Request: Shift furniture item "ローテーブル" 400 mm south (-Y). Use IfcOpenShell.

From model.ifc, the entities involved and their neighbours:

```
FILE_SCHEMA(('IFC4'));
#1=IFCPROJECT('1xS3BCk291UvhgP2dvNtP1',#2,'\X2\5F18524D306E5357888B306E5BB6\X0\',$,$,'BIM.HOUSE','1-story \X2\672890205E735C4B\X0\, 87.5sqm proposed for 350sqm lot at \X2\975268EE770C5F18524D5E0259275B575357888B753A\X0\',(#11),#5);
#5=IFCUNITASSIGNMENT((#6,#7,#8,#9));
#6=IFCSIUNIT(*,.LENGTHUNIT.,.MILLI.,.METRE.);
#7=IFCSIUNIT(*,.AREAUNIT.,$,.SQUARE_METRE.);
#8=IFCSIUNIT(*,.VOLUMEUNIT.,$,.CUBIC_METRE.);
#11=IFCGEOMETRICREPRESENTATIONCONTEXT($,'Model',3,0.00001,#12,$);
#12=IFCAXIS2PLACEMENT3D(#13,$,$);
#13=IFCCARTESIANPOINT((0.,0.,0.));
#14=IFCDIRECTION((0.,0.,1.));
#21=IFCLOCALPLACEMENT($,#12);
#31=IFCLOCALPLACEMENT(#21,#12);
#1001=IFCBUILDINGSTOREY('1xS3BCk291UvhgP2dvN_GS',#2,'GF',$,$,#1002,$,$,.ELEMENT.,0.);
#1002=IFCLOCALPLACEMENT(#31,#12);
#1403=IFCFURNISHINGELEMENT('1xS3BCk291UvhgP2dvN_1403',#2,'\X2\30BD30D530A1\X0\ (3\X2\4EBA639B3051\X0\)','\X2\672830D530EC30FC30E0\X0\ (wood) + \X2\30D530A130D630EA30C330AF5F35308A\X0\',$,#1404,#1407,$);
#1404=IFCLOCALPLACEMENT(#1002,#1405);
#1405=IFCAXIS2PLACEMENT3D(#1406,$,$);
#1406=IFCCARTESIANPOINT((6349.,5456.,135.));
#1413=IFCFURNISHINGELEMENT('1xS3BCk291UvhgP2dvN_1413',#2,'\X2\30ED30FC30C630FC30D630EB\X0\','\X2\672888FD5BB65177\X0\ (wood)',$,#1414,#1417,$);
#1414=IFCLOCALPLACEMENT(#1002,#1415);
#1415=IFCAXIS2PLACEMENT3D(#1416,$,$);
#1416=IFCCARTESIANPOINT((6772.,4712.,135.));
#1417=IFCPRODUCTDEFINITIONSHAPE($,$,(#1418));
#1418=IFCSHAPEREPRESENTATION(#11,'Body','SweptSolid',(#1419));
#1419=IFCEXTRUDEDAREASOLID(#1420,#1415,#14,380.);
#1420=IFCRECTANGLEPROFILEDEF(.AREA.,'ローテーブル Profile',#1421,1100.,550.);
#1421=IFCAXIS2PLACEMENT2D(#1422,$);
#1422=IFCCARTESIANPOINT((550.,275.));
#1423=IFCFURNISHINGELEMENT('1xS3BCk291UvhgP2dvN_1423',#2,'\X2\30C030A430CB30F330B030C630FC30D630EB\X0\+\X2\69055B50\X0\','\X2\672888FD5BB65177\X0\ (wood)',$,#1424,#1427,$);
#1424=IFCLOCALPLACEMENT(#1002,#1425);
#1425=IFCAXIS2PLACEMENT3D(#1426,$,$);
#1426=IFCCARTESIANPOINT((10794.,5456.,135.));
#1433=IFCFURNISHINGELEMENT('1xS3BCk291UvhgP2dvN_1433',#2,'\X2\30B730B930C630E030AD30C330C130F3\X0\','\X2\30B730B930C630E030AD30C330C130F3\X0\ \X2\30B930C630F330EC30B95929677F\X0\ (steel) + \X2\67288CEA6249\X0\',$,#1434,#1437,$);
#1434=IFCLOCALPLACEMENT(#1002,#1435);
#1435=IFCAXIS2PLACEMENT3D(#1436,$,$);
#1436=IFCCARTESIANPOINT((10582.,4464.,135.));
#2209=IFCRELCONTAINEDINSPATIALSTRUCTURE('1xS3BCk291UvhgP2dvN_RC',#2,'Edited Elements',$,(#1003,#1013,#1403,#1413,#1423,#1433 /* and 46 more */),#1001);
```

```python
import ifcopenshell
import ifcopenshell.api.geometry
import ifcopenshell.util.placement

model = ifcopenshell.open("model.ifc")

item = model.by_guid("1xS3BCk291UvhgP2dvN_1413")
matrix = ifcopenshell.util.placement.get_local_placement(item.ObjectPlacement)
matrix[1, 3] -= 400.0
ifcopenshell.api.geometry.edit_object_placement(model, product=item, matrix=matrix, is_si=False)

print(ifcopenshell.util.placement.get_local_placement(item.ObjectPlacement).round(3) + 0.0)

model.write("model_v2.ifc")
```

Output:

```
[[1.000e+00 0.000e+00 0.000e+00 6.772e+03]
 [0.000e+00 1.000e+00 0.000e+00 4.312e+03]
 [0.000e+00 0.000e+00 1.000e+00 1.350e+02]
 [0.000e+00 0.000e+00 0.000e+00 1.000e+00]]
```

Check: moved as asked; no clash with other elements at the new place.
